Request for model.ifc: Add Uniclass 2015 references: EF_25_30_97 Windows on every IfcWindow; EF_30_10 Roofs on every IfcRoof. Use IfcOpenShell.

First a look at what the model holds.

```python
import ifcopenshell

model = ifcopenshell.open("model.ifc")
print(model.schema)
print("classifications:", [c.Name for c in model.by_type("IfcClassification")])
for ifc_class in ("IfcDoor", "IfcRoof", "IfcStair", "IfcWall", "IfcWindow"):
    print(ifc_class, len(model.by_type(ifc_class)))
```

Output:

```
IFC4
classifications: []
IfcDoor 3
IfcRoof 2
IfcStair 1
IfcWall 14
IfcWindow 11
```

```python
import ifcopenshell
import ifcopenshell.api.classification

model = ifcopenshell.open("model.ifc")

system = ifcopenshell.api.classification.add_classification(model, classification="Uniclass 2015")

codes = {
    "IfcWindow": ("EF_25_30_97", "Windows"),
    "IfcRoof": ("EF_30_10", "Roofs"),
}
for ifc_class, (code, name) in codes.items():
    products = model.by_type(ifc_class)
    ifcopenshell.api.classification.add_reference(
        model, products=products, classification=system, identification=code, name=name
    )
    print(code, len(products))

model.write("model_v2.ifc")
```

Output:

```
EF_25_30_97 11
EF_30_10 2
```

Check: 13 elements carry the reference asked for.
